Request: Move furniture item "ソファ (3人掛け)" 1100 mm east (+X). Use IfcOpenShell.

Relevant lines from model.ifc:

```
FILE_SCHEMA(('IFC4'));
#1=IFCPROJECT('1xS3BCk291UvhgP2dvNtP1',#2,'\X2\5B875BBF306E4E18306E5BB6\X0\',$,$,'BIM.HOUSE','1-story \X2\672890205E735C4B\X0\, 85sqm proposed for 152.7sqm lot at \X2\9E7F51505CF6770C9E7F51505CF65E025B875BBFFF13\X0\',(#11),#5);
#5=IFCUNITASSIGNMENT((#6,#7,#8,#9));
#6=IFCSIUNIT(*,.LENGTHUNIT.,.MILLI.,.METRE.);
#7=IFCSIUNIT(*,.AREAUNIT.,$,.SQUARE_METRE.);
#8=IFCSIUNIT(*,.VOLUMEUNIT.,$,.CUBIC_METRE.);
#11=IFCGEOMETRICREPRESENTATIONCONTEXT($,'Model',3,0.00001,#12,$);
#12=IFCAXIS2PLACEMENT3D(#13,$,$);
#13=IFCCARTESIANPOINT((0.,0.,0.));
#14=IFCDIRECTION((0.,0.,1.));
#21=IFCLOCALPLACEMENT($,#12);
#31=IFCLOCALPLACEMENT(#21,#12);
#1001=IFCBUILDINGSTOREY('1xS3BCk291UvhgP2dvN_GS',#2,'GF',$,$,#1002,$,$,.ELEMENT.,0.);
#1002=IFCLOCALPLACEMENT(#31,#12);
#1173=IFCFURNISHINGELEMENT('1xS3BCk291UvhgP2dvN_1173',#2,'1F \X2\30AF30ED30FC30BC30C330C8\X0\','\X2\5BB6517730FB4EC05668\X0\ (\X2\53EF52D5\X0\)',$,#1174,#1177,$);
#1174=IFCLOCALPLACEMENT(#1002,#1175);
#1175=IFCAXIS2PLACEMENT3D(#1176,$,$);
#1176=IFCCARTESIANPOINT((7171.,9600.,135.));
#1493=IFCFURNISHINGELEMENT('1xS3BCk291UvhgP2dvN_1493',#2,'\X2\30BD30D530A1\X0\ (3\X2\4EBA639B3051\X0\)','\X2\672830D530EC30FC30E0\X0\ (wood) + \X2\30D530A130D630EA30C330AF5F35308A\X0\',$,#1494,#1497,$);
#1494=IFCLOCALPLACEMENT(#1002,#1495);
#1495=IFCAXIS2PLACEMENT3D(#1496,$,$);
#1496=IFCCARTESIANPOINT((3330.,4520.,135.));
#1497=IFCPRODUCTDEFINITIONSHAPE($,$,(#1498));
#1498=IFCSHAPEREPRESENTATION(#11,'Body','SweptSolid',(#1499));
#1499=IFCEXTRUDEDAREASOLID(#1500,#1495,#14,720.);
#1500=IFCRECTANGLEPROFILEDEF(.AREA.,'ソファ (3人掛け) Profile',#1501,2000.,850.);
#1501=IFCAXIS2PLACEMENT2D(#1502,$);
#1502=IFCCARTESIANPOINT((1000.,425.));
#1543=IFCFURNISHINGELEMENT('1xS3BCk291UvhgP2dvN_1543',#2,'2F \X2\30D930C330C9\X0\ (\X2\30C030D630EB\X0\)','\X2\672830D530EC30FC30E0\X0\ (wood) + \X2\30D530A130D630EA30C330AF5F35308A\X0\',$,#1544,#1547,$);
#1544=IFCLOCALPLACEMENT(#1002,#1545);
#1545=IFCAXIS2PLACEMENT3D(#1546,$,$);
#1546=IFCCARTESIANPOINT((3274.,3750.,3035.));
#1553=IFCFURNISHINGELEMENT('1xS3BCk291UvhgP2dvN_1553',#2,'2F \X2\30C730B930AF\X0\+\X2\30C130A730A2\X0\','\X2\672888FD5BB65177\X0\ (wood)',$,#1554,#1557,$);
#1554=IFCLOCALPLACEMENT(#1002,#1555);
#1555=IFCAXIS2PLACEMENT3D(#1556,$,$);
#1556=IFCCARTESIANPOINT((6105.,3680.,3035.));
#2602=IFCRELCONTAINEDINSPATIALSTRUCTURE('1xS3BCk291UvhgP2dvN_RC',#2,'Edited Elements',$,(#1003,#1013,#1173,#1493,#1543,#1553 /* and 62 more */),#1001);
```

```python
import ifcopenshell
import ifcopenshell.api.geometry
import ifcopenshell.util.placement

model = ifcopenshell.open("model.ifc")

item = model.by_guid("1xS3BCk291UvhgP2dvN_1493")
matrix = ifcopenshell.util.placement.get_local_placement(item.ObjectPlacement)
matrix[0, 3] += 1100.0
ifcopenshell.api.geometry.edit_object_placement(model, product=item, matrix=matrix, is_si=False)

print(ifcopenshell.util.placement.get_local_placement(item.ObjectPlacement).round(3) + 0.0)

model.write("model-out.ifc")
```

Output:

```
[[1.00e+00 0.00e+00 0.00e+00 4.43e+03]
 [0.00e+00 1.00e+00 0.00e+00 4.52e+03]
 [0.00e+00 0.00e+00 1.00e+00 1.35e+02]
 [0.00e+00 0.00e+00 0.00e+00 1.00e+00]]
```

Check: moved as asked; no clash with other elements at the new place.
